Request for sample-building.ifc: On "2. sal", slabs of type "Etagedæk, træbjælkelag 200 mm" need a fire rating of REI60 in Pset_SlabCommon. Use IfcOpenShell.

First a look at what the model holds.

```python
import ifcopenshell
import ifcopenshell.util.element

model = ifcopenshell.open("sample-building.ifc")
print(model.schema)
storey = next(s for s in model.by_type("IfcBuildingStorey") if s.Name == "2. sal")
slabs = [e for e in ifcopenshell.util.element.get_decomposition(storey) if e.is_a("IfcSlab")]
seen = {}
for e in slabs:
    element_type = ifcopenshell.util.element.get_type(e)
    key = (element_type.Name if element_type != e and element_type else None, ifcopenshell.util.element.get_pset(e, "Pset_SlabCommon", "FireRating"))
    seen[key] = seen.get(key, 0) + 1
for (name, value), count in sorted(seen.items(), key=str):
    print(count, "x", name, "|", value)
```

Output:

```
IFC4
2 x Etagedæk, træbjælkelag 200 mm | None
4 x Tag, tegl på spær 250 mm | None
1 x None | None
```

```python
import ifcopenshell
import ifcopenshell.api.pset
import ifcopenshell.util.element

model = ifcopenshell.open("sample-building.ifc")

storey = next(s for s in model.by_type("IfcBuildingStorey") if s.Name == "2. sal")
slabs = [e for e in ifcopenshell.util.element.get_decomposition(storey) if e.is_a("IfcSlab")]

count = 0
for e in slabs:
    element_type = ifcopenshell.util.element.get_type(e)
    if element_type in (None, e) or element_type.Name != "Etagedæk, træbjælkelag 200 mm":
        continue
    found = ifcopenshell.util.element.get_pset(e, "Pset_SlabCommon", should_inherit=False)
    if found:
        pset = model.by_id(found["id"])
        if len(ifcopenshell.util.element.get_elements_by_pset(pset)) > 1:
            pset = ifcopenshell.api.pset.unshare_pset(model, products=[e], pset=pset)[0]
    else:
        pset = ifcopenshell.api.pset.add_pset(model, product=e, name="Pset_SlabCommon")
    ifcopenshell.api.pset.edit_pset(model, pset=pset, properties={"FireRating": "REI60"})
    count += 1

print(count, "slabs updated")

model.write("sample-building_edited.ifc")
```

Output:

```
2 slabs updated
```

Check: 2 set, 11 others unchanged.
